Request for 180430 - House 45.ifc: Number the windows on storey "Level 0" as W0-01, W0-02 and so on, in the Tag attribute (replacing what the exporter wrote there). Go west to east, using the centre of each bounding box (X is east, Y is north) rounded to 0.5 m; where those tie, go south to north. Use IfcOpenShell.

First a look at what the model holds.

```python
import ifcopenshell
import ifcopenshell.util.element
import ifcopenshell.util.placement

model = ifcopenshell.open("180430 - House 45.ifc")
print(model.schema)
storey = next(s for s in model.by_type("IfcBuildingStorey") if s.Name == "Level 0")
windows = [e for e in ifcopenshell.util.element.get_decomposition(storey) if e.is_a("IfcWindow")]
for e in sorted(windows, key=lambda e: e.id()):
    origin = ifcopenshell.util.placement.get_local_placement(e.ObjectPlacement)[:3, 3]
    print(e.id(), e.Tag, e.Name, origin.round(2) + 0.0, sep=" | ")
```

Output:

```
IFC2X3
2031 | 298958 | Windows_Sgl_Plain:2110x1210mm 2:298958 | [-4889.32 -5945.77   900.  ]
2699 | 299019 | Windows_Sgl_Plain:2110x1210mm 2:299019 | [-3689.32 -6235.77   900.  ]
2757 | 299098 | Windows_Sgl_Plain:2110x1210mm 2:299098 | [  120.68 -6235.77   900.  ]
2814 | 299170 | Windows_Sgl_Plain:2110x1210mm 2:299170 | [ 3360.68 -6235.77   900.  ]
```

```python
import ifcopenshell
import ifcopenshell.geom
import ifcopenshell.util.element
import ifcopenshell.util.shape

model = ifcopenshell.open("180430 - House 45.ifc")
settings = ifcopenshell.geom.settings()
settings.set("use-world-coords", True)


def centre(element):
    shape = ifcopenshell.geom.create_shape(settings, element)
    return ifcopenshell.util.shape.get_bbox_centroid(shape.geometry)


storey = next(s for s in model.by_type("IfcBuildingStorey") if s.Name == "Level 0")
windows = [e for e in ifcopenshell.util.element.get_decomposition(storey) if e.is_a("IfcWindow")]

# Insertion points can sit at a corner or the storey origin, so sort by the geometry (in metres).
centres = {e: centre(e) for e in windows}
windows.sort(key=lambda e: (round(centres[e][0] / 0.5), centres[e][1]))

for i, e in enumerate(windows, start=1):
    number = f"W0-{i:02d}"
    e.Tag = number
    print(e.id(), number)

model.write("180430 - House 45_v2.ifc")
```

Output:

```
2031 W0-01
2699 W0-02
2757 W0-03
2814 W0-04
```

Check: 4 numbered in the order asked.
